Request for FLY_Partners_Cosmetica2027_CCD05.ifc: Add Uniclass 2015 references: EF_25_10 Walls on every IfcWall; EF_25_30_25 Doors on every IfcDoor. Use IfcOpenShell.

First a look at what the model holds.

```python
import ifcopenshell

model = ifcopenshell.open("FLY_Partners_Cosmetica2027_CCD05.ifc")
print(model.schema)
print("classifications:", [c.Name for c in model.by_type("IfcClassification")])
for ifc_class in ("IfcDoor", "IfcRoof", "IfcStair", "IfcWall", "IfcWindow"):
    print(ifc_class, len(model.by_type(ifc_class)))
```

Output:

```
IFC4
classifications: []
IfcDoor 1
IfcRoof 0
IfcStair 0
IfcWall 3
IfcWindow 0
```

```python
import ifcopenshell
import ifcopenshell.api.classification

model = ifcopenshell.open("FLY_Partners_Cosmetica2027_CCD05.ifc")

system = ifcopenshell.api.classification.add_classification(model, classification="Uniclass 2015")

codes = {
    "IfcWall": ("EF_25_10", "Walls"),
    "IfcDoor": ("EF_25_30_25", "Doors"),
}
for ifc_class, (code, name) in codes.items():
    products = model.by_type(ifc_class)
    ifcopenshell.api.classification.add_reference(
        model, products=products, classification=system, identification=code, name=name
    )
    print(code, len(products))

model.write("FLY_Partners_Cosmetica2027_CCD05-out.ifc")
```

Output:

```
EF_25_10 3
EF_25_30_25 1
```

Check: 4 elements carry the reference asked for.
